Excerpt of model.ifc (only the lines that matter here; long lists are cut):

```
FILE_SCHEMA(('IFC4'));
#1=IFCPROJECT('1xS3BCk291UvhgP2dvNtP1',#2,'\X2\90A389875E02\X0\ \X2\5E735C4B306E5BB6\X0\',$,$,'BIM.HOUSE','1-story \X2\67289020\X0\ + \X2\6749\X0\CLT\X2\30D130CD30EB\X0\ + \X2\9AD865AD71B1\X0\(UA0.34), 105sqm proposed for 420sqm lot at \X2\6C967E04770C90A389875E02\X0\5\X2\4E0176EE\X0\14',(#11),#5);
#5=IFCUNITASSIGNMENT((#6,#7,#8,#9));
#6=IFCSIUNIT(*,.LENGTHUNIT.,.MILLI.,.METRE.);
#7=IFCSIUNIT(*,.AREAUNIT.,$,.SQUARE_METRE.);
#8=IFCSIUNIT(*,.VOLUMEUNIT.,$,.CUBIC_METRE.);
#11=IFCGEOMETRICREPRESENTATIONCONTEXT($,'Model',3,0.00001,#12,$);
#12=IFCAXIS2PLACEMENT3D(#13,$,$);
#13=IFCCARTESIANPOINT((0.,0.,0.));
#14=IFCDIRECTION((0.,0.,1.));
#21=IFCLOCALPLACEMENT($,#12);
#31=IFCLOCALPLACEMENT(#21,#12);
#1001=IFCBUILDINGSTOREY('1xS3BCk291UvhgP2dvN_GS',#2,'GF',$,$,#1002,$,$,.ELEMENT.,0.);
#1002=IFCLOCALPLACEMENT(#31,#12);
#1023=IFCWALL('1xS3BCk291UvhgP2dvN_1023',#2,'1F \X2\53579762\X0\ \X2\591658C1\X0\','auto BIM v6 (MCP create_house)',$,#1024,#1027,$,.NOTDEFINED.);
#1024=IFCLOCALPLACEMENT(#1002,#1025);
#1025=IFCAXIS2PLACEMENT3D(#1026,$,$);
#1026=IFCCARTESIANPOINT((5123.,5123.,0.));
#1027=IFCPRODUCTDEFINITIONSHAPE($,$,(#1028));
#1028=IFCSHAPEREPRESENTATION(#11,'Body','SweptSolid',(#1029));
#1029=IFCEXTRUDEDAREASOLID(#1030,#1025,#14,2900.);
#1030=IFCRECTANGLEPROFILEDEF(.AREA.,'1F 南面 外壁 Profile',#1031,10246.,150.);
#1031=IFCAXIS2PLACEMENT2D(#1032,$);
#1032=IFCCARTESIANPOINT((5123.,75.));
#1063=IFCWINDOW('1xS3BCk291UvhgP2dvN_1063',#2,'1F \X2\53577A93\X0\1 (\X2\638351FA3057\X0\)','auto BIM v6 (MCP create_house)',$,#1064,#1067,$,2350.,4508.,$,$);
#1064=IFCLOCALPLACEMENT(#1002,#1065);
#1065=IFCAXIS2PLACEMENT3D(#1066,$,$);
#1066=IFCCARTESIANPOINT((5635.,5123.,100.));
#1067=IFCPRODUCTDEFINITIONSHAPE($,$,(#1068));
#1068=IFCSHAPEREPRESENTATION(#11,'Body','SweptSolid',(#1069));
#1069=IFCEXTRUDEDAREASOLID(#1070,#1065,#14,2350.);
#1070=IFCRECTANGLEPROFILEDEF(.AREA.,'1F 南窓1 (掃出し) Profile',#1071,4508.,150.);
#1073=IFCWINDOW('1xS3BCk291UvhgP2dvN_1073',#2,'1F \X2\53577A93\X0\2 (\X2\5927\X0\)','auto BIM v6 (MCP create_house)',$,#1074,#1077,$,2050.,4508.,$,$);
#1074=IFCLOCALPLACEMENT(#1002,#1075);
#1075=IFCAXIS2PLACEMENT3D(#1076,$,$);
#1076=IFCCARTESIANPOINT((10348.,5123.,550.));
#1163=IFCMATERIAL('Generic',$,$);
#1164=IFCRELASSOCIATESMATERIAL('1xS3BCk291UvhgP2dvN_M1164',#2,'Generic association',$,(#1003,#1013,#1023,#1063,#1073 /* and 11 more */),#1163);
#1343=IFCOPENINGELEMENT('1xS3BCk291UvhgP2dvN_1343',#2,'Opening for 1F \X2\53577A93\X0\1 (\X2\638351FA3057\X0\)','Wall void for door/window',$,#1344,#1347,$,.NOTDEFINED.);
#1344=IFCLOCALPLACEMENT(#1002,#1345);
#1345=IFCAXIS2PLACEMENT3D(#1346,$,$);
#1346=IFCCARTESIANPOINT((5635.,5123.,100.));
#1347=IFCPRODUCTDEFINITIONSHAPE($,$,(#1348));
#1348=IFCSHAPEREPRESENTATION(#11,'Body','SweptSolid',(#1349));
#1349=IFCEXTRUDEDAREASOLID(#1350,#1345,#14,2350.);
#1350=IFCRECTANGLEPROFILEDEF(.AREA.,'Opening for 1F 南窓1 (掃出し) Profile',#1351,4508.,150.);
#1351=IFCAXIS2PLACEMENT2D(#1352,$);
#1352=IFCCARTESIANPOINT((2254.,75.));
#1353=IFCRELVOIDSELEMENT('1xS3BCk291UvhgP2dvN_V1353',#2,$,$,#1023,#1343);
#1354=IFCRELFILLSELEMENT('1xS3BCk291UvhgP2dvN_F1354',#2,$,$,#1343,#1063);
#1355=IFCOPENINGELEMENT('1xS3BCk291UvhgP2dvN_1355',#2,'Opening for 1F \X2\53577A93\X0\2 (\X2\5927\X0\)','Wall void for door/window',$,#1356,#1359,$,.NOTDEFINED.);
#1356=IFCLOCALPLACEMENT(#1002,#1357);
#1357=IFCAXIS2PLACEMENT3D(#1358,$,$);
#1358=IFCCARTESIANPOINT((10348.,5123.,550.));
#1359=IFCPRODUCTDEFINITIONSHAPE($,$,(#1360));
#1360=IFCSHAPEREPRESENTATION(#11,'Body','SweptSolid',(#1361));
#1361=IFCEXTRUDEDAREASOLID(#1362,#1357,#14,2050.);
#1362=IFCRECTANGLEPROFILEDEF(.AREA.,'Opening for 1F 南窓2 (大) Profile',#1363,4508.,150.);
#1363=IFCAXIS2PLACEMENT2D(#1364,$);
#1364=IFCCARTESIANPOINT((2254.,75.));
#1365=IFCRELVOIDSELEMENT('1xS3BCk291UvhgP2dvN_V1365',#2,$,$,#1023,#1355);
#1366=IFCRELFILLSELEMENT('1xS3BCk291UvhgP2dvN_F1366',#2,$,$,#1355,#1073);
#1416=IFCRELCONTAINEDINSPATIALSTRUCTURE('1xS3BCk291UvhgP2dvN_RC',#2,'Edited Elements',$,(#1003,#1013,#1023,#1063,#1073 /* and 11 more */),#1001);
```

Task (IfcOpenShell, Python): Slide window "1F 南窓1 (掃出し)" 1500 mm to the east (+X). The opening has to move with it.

```python
import ifcopenshell
import ifcopenshell.api.geometry
import ifcopenshell.util.placement
import ifcopenshell.util.unit

model = ifcopenshell.open("model.ifc")
unit_scale = ifcopenshell.util.unit.calculate_unit_scale(model)

window = model.by_guid("1xS3BCk291UvhgP2dvN_1063")
opening = window.FillsVoids[0].RelatingOpeningElement
wall = opening.VoidsElements[0].RelatingBuildingElement

wall_matrix = ifcopenshell.util.placement.get_local_placement(wall.ObjectPlacement)
shift = wall_matrix[:3, 0] * 1.5 / unit_scale
before = ifcopenshell.util.placement.get_local_placement(window.ObjectPlacement)[:3, 3].copy()

# The window is not placed relative to its opening, so move both.
for product in (opening, window):
    matrix = ifcopenshell.util.placement.get_local_placement(product.ObjectPlacement)
    matrix[:3, 3] += shift
    ifcopenshell.api.geometry.edit_object_placement(model, product=product, matrix=matrix, is_si=False)

after = ifcopenshell.util.placement.get_local_placement(window.ObjectPlacement)[:3, 3]
print("window moved by", (after - before).round(3) + 0.0)

model.write("model-out.ifc")
```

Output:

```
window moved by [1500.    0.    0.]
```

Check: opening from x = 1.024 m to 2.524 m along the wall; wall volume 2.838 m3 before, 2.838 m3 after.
